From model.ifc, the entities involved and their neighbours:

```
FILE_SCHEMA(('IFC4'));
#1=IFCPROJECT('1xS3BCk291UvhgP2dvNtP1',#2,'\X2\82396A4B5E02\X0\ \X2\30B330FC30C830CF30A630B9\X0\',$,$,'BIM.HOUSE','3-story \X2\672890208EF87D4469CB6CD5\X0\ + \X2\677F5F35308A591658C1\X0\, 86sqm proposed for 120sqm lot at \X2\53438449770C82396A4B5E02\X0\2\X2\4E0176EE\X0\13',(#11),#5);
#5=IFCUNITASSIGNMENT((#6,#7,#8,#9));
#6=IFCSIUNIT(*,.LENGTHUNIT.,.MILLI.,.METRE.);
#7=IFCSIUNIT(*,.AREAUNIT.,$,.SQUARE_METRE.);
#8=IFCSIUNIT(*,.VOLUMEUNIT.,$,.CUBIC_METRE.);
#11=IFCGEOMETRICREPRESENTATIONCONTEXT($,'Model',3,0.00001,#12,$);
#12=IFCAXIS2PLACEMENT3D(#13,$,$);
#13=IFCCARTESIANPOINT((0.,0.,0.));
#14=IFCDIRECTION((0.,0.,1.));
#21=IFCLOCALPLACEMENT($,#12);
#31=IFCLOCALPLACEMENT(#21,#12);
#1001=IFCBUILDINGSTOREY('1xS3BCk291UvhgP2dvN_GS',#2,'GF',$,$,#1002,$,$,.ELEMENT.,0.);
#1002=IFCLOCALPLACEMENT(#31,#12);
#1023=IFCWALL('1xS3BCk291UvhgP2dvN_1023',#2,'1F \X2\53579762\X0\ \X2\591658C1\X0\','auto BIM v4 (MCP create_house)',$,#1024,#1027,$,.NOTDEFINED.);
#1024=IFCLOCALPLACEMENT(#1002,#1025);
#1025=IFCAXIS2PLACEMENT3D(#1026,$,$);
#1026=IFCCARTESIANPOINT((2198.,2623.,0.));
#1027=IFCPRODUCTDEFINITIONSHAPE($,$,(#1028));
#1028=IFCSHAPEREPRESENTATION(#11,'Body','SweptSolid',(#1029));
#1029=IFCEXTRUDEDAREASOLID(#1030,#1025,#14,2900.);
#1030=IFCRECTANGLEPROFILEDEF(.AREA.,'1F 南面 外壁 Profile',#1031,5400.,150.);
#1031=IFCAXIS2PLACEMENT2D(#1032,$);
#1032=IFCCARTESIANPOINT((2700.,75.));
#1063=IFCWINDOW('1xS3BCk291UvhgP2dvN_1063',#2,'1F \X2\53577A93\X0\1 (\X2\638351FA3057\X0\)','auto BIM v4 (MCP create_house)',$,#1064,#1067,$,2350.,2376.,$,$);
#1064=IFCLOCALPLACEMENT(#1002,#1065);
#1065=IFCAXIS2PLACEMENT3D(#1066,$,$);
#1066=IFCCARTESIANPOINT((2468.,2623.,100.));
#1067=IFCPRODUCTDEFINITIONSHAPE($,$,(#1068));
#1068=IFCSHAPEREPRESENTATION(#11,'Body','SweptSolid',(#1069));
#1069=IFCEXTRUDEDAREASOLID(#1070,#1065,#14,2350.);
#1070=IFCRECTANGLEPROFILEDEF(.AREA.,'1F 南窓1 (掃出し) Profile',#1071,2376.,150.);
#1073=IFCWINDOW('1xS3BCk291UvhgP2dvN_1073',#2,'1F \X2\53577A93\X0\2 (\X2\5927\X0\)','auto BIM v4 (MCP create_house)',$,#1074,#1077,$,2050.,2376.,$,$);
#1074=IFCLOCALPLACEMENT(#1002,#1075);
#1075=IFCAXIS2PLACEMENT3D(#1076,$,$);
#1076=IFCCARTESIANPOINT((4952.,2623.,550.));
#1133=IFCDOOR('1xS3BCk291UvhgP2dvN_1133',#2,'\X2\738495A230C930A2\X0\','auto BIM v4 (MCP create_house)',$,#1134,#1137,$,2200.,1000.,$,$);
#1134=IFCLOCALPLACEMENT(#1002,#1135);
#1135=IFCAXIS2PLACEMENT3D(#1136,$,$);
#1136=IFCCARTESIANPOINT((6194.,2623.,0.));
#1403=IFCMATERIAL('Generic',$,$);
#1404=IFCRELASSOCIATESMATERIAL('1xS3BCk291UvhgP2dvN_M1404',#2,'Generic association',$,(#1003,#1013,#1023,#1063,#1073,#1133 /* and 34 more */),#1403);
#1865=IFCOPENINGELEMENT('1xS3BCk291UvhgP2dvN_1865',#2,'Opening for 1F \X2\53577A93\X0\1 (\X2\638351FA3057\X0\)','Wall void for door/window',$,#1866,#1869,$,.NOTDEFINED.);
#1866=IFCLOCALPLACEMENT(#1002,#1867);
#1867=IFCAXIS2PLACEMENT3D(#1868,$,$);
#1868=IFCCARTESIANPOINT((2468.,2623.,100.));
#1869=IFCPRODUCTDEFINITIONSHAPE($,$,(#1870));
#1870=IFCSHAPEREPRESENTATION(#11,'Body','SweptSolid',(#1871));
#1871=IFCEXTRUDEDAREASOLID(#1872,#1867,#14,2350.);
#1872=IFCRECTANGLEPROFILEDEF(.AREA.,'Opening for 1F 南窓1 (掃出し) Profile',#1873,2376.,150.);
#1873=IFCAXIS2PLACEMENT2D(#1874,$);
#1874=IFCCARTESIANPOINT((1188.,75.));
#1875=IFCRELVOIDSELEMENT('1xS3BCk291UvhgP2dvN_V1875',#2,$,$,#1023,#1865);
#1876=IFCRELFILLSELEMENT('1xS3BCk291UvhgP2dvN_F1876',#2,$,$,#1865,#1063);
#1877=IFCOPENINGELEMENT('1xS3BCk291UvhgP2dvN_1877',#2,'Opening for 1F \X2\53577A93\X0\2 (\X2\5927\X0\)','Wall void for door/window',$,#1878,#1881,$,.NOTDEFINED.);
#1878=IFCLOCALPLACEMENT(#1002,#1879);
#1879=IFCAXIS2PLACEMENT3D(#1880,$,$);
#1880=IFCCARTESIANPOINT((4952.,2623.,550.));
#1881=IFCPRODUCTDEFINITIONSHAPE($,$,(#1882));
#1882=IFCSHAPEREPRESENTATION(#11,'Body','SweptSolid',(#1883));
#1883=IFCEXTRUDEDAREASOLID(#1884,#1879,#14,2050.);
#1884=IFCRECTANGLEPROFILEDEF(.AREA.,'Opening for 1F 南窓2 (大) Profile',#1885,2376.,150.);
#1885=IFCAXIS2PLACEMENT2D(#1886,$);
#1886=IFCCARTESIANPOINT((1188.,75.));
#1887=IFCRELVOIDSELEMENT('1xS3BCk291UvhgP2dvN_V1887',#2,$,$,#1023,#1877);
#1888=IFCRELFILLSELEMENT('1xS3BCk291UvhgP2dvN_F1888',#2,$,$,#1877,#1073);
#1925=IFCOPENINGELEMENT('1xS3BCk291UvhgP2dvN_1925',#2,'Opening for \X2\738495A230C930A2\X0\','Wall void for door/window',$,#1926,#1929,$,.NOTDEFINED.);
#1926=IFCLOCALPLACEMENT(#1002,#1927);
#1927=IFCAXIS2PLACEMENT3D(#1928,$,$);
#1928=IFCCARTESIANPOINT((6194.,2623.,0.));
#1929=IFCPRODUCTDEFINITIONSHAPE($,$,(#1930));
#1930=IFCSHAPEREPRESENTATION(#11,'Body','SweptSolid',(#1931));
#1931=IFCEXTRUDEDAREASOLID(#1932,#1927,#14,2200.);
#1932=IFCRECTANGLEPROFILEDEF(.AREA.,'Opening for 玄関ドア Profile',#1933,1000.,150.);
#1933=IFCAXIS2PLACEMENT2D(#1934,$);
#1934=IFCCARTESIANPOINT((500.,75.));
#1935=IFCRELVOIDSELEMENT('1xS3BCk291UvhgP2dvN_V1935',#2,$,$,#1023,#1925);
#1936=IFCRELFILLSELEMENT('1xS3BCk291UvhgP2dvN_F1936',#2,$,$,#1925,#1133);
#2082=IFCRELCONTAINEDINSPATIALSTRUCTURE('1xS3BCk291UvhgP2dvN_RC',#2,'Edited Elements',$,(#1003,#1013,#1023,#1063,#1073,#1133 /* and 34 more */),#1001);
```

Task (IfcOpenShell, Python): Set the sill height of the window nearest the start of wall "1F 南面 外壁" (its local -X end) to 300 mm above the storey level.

```python
import numpy as np
import ifcopenshell
import ifcopenshell.api.geometry
import ifcopenshell.geom
import ifcopenshell.util.element
import ifcopenshell.util.placement
import ifcopenshell.util.shape
import ifcopenshell.util.unit

model = ifcopenshell.open("model.ifc")
unit_scale = ifcopenshell.util.unit.calculate_unit_scale(model)

window = model.by_id(1063)
opening = window.FillsVoids[0].RelatingOpeningElement
storey = ifcopenshell.util.element.get_container(window, ifc_class="IfcBuildingStorey")
level = ifcopenshell.util.placement.get_local_placement(storey.ObjectPlacement)[2, 3]

# The opening's origin need not be at the sill, so measure its lowest point.
shape = ifcopenshell.geom.create_shape(ifcopenshell.geom.settings(), opening)
bottom = ifcopenshell.util.shape.get_shape_bottom_elevation(shape, shape.geometry) / unit_scale
dz = level + 0.3 / unit_scale - bottom

shift = np.array([0.0, 0.0, dz])
# The window is not placed relative to its opening, so move both.
for product in (opening, window):
    matrix = ifcopenshell.util.placement.get_local_placement(product.ObjectPlacement)
    matrix[:3, 3] += shift
    ifcopenshell.api.geometry.edit_object_placement(model, product=product, matrix=matrix, is_si=False)

print(f"moved by {dz * unit_scale:+.3f} m")

model.write("model-out.ifc")
```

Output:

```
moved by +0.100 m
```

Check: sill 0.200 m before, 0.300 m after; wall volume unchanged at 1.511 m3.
